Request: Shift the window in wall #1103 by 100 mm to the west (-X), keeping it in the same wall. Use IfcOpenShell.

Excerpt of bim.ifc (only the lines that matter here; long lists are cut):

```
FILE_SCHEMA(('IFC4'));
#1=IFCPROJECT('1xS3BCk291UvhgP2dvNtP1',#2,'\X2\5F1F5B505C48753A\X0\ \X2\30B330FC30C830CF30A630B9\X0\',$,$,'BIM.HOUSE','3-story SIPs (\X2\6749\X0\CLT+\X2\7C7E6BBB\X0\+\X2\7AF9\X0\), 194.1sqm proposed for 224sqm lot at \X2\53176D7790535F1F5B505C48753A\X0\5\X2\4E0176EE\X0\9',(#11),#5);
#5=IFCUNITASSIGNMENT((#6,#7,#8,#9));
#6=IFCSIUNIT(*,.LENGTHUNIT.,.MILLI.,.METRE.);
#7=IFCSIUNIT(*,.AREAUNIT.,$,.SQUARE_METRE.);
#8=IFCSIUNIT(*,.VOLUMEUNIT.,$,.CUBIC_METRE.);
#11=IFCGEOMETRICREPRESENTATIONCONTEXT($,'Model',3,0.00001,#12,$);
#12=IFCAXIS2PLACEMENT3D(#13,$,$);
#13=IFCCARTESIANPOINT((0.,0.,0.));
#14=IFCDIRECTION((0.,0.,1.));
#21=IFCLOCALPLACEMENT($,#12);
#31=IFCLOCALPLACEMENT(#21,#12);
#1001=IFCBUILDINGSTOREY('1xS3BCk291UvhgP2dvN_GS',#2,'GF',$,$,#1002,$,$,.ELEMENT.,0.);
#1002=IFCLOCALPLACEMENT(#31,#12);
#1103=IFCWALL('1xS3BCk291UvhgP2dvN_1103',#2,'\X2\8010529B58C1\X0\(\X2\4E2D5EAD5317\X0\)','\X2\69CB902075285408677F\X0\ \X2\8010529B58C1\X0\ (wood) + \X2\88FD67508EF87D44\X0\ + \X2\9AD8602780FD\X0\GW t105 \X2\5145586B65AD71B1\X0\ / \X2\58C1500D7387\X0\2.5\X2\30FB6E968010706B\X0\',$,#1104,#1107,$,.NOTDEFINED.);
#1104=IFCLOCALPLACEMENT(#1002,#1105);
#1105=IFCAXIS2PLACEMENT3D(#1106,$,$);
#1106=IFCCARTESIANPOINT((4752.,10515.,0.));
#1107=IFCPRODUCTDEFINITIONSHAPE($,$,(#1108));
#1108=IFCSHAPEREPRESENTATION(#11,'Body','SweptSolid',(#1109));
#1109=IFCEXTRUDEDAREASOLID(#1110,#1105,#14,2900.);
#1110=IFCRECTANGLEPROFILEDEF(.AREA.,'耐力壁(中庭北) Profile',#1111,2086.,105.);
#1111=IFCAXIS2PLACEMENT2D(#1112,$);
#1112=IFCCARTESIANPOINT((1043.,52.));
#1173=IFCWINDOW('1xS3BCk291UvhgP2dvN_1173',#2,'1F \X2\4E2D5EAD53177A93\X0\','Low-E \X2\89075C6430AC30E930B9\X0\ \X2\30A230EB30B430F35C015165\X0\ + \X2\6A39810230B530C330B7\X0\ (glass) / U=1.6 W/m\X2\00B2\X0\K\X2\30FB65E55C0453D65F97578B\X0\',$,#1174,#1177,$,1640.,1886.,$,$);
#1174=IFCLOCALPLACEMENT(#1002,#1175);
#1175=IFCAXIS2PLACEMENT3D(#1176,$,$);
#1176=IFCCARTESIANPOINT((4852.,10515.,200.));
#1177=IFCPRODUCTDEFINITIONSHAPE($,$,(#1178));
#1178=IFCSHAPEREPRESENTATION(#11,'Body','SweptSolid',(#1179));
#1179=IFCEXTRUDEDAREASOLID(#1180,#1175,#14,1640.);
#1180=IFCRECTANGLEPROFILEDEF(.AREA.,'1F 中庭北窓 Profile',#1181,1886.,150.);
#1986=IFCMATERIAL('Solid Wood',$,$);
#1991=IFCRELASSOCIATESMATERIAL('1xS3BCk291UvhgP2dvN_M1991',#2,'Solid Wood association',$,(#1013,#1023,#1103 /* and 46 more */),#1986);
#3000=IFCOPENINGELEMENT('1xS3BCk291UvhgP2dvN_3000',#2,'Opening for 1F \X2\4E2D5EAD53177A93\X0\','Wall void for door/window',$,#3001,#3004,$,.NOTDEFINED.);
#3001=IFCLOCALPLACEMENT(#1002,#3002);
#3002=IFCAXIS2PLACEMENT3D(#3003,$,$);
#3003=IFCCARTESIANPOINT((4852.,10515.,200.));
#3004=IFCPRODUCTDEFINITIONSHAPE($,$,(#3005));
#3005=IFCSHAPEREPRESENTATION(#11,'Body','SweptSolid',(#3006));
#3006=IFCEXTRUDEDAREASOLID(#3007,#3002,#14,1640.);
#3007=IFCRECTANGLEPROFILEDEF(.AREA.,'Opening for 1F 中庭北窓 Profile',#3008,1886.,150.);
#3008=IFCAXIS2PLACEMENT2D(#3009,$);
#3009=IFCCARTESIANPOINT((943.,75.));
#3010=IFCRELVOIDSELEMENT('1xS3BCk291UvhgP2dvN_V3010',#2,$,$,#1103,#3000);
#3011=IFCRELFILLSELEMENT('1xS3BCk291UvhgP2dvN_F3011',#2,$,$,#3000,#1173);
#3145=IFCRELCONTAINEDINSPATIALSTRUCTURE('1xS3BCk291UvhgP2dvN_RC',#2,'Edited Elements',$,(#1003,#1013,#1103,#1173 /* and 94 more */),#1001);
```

```python
import ifcopenshell
import ifcopenshell.api.geometry
import ifcopenshell.util.placement
import ifcopenshell.util.unit

model = ifcopenshell.open("bim.ifc")
unit_scale = ifcopenshell.util.unit.calculate_unit_scale(model)

window = model.by_guid("1xS3BCk291UvhgP2dvN_1173")
opening = window.FillsVoids[0].RelatingOpeningElement
wall = opening.VoidsElements[0].RelatingBuildingElement

wall_matrix = ifcopenshell.util.placement.get_local_placement(wall.ObjectPlacement)
shift = wall_matrix[:3, 0] * -0.1 / unit_scale
before = ifcopenshell.util.placement.get_local_placement(window.ObjectPlacement)[:3, 3].copy()

# The window is not placed relative to its opening, so move both.
for product in (opening, window):
    matrix = ifcopenshell.util.placement.get_local_placement(product.ObjectPlacement)
    matrix[:3, 3] += shift
    ifcopenshell.api.geometry.edit_object_placement(model, product=product, matrix=matrix, is_si=False)

after = ifcopenshell.util.placement.get_local_placement(window.ObjectPlacement)[:3, 3]
print("window moved by", (after - before).round(3) + 0.0)

model.write("bim_rev.ifc")
```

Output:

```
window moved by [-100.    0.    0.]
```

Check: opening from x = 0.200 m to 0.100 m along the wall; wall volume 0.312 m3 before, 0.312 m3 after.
